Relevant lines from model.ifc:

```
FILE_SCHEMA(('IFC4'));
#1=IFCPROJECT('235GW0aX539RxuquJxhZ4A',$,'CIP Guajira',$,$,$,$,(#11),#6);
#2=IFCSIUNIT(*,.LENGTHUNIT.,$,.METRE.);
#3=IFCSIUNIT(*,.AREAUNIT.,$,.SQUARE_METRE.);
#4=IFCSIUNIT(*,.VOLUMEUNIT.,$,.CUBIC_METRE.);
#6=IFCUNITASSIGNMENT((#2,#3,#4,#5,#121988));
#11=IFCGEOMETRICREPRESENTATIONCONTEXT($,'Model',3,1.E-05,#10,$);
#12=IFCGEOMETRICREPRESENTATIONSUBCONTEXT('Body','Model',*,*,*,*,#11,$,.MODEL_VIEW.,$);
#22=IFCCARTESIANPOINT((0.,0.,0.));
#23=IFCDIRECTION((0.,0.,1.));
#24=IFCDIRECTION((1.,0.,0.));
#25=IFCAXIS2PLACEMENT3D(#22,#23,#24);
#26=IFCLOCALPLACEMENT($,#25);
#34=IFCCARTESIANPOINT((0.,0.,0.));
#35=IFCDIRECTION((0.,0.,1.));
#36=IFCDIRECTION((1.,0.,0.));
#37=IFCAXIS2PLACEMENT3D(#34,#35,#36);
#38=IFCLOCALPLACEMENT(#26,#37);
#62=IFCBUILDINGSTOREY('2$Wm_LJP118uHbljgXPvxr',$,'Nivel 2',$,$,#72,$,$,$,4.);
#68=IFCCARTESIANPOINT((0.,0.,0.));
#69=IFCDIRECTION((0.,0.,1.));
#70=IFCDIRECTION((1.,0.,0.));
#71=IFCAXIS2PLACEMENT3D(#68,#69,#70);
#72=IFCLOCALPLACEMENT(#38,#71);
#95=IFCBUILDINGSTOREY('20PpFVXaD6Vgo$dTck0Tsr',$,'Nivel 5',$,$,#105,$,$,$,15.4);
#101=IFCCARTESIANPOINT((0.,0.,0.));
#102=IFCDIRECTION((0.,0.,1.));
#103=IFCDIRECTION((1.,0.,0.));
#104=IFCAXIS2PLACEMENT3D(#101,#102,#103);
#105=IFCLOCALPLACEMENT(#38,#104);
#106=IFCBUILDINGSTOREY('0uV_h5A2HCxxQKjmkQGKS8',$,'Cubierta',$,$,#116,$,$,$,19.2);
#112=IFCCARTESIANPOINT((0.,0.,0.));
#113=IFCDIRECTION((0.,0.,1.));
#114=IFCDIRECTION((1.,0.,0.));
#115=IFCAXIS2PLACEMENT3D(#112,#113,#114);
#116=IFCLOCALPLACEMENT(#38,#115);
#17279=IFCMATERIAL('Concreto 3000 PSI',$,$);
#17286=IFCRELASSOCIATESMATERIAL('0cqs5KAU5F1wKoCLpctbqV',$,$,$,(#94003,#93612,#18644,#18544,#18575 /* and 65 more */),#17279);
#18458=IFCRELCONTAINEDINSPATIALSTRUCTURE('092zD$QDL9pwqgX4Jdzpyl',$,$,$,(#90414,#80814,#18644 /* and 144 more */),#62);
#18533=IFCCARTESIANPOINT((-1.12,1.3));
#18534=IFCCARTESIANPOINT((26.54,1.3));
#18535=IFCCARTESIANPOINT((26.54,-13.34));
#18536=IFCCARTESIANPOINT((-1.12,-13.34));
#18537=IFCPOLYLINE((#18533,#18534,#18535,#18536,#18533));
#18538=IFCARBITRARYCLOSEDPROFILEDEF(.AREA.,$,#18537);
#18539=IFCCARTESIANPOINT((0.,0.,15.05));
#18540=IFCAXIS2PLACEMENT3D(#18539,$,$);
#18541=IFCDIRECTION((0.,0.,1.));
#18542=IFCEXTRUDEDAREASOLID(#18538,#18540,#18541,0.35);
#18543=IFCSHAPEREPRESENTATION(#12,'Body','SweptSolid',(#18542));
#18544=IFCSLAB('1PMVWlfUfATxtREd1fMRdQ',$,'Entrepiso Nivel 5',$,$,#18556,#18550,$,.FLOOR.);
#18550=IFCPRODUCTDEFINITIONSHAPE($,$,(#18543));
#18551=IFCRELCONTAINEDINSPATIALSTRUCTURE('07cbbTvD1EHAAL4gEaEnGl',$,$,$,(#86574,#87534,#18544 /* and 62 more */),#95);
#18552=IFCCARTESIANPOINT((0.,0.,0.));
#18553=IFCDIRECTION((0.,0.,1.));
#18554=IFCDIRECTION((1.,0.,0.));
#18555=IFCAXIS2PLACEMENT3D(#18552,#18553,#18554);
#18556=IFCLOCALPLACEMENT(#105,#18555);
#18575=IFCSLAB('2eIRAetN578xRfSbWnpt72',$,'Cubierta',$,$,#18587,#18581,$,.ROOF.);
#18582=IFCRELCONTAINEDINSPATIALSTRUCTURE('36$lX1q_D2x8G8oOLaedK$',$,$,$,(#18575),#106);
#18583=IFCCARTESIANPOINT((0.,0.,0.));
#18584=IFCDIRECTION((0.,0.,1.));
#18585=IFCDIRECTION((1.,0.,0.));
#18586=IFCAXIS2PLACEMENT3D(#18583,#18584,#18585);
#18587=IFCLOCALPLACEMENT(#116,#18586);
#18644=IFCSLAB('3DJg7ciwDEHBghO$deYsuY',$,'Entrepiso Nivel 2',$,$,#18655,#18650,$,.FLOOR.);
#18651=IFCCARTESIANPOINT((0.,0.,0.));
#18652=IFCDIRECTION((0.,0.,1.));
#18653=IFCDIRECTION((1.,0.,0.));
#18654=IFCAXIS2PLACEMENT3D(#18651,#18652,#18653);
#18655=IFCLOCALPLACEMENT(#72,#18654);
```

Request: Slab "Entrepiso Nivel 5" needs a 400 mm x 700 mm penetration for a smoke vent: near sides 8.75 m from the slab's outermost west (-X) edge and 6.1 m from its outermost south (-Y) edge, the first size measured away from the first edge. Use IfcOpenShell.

```python
import numpy as np
import ifcopenshell
import ifcopenshell.api.feature
import ifcopenshell.api.geometry
import ifcopenshell.api.root
import ifcopenshell.geom
import ifcopenshell.util.placement
import ifcopenshell.util.representation
import ifcopenshell.util.shape
import ifcopenshell.util.unit

model = ifcopenshell.open("model.ifc")
unit_scale = ifcopenshell.util.unit.calculate_unit_scale(model)
settings = ifcopenshell.geom.settings()


def volume(element):
    """Net volume in cubic metres, openings subtracted."""
    shape = ifcopenshell.geom.create_shape(settings, element)
    return ifcopenshell.util.shape.get_volume(shape.geometry)


slab = model.by_guid("1PMVWlfUfATxtREd1fMRdQ")
before = volume(slab)

# Extent in the slab's own axes, in metres. The edges named are its -X and -Y sides.
slab_shape = ifcopenshell.geom.create_shape(settings, slab)
vertices = ifcopenshell.util.shape.get_vertices(slab_shape.geometry)
x_min, y_min, bottom = vertices.min(axis=0)
top = vertices[:, 2].max()

opening = ifcopenshell.api.root.create_entity(model, ifc_class="IfcOpeningElement", name="Smoke vent opening", predefined_type="OPENING")
context = ifcopenshell.util.representation.get_context(model, "Model", "Body", "MODEL_VIEW")
width, depth = 0.4, 0.7
outline = [(0.0, 0.0), (width, 0.0), (width, depth), (0.0, depth), (0.0, 0.0)]
# Overshoot both faces by 50 mm so the cut is clean.
shape = ifcopenshell.api.geometry.add_slab_representation(
    model, context=context, depth=top - bottom + 0.1, polyline=outline
)
ifcopenshell.api.geometry.assign_representation(model, product=opening, representation=shape)

matrix = ifcopenshell.util.placement.get_local_placement(slab.ObjectPlacement)
matrix[:, 3] = matrix @ np.append(np.array([x_min + 8.75, y_min + 6.1, bottom - 0.05]) / unit_scale, 1.0)
ifcopenshell.api.geometry.edit_object_placement(model, product=opening, matrix=matrix, is_si=False)
ifcopenshell.api.feature.add_feature(model, feature=opening, element=slab)

after = volume(slab)

print(f"slab volume {before:.3f} -> {after:.3f} m3")

model.write("model-out.ifc")
```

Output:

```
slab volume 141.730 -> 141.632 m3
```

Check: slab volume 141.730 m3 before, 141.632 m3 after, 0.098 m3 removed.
